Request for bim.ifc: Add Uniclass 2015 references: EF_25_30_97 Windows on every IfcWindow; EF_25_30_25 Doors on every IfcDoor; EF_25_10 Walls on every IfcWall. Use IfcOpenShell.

First a look at what the model holds.

```python
import ifcopenshell

model = ifcopenshell.open("bim.ifc")
print(model.schema)
print("classifications:", [c.Name for c in model.by_type("IfcClassification")])
for ifc_class in ("IfcDoor", "IfcRoof", "IfcStair", "IfcWall", "IfcWindow"):
    print(ifc_class, len(model.by_type(ifc_class)))
```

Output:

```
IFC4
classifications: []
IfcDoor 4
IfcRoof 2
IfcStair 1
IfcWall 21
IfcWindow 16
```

```python
import ifcopenshell
import ifcopenshell.api.classification

model = ifcopenshell.open("bim.ifc")

system = ifcopenshell.api.classification.add_classification(model, classification="Uniclass 2015")

codes = {
    "IfcWindow": ("EF_25_30_97", "Windows"),
    "IfcDoor": ("EF_25_30_25", "Doors"),
    "IfcWall": ("EF_25_10", "Walls"),
}
for ifc_class, (code, name) in codes.items():
    products = model.by_type(ifc_class)
    ifcopenshell.api.classification.add_reference(
        model, products=products, classification=system, identification=code, name=name
    )
    print(code, len(products))

model.write("bim-out.ifc")
```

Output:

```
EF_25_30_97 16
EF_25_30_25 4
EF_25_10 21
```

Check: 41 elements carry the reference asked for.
